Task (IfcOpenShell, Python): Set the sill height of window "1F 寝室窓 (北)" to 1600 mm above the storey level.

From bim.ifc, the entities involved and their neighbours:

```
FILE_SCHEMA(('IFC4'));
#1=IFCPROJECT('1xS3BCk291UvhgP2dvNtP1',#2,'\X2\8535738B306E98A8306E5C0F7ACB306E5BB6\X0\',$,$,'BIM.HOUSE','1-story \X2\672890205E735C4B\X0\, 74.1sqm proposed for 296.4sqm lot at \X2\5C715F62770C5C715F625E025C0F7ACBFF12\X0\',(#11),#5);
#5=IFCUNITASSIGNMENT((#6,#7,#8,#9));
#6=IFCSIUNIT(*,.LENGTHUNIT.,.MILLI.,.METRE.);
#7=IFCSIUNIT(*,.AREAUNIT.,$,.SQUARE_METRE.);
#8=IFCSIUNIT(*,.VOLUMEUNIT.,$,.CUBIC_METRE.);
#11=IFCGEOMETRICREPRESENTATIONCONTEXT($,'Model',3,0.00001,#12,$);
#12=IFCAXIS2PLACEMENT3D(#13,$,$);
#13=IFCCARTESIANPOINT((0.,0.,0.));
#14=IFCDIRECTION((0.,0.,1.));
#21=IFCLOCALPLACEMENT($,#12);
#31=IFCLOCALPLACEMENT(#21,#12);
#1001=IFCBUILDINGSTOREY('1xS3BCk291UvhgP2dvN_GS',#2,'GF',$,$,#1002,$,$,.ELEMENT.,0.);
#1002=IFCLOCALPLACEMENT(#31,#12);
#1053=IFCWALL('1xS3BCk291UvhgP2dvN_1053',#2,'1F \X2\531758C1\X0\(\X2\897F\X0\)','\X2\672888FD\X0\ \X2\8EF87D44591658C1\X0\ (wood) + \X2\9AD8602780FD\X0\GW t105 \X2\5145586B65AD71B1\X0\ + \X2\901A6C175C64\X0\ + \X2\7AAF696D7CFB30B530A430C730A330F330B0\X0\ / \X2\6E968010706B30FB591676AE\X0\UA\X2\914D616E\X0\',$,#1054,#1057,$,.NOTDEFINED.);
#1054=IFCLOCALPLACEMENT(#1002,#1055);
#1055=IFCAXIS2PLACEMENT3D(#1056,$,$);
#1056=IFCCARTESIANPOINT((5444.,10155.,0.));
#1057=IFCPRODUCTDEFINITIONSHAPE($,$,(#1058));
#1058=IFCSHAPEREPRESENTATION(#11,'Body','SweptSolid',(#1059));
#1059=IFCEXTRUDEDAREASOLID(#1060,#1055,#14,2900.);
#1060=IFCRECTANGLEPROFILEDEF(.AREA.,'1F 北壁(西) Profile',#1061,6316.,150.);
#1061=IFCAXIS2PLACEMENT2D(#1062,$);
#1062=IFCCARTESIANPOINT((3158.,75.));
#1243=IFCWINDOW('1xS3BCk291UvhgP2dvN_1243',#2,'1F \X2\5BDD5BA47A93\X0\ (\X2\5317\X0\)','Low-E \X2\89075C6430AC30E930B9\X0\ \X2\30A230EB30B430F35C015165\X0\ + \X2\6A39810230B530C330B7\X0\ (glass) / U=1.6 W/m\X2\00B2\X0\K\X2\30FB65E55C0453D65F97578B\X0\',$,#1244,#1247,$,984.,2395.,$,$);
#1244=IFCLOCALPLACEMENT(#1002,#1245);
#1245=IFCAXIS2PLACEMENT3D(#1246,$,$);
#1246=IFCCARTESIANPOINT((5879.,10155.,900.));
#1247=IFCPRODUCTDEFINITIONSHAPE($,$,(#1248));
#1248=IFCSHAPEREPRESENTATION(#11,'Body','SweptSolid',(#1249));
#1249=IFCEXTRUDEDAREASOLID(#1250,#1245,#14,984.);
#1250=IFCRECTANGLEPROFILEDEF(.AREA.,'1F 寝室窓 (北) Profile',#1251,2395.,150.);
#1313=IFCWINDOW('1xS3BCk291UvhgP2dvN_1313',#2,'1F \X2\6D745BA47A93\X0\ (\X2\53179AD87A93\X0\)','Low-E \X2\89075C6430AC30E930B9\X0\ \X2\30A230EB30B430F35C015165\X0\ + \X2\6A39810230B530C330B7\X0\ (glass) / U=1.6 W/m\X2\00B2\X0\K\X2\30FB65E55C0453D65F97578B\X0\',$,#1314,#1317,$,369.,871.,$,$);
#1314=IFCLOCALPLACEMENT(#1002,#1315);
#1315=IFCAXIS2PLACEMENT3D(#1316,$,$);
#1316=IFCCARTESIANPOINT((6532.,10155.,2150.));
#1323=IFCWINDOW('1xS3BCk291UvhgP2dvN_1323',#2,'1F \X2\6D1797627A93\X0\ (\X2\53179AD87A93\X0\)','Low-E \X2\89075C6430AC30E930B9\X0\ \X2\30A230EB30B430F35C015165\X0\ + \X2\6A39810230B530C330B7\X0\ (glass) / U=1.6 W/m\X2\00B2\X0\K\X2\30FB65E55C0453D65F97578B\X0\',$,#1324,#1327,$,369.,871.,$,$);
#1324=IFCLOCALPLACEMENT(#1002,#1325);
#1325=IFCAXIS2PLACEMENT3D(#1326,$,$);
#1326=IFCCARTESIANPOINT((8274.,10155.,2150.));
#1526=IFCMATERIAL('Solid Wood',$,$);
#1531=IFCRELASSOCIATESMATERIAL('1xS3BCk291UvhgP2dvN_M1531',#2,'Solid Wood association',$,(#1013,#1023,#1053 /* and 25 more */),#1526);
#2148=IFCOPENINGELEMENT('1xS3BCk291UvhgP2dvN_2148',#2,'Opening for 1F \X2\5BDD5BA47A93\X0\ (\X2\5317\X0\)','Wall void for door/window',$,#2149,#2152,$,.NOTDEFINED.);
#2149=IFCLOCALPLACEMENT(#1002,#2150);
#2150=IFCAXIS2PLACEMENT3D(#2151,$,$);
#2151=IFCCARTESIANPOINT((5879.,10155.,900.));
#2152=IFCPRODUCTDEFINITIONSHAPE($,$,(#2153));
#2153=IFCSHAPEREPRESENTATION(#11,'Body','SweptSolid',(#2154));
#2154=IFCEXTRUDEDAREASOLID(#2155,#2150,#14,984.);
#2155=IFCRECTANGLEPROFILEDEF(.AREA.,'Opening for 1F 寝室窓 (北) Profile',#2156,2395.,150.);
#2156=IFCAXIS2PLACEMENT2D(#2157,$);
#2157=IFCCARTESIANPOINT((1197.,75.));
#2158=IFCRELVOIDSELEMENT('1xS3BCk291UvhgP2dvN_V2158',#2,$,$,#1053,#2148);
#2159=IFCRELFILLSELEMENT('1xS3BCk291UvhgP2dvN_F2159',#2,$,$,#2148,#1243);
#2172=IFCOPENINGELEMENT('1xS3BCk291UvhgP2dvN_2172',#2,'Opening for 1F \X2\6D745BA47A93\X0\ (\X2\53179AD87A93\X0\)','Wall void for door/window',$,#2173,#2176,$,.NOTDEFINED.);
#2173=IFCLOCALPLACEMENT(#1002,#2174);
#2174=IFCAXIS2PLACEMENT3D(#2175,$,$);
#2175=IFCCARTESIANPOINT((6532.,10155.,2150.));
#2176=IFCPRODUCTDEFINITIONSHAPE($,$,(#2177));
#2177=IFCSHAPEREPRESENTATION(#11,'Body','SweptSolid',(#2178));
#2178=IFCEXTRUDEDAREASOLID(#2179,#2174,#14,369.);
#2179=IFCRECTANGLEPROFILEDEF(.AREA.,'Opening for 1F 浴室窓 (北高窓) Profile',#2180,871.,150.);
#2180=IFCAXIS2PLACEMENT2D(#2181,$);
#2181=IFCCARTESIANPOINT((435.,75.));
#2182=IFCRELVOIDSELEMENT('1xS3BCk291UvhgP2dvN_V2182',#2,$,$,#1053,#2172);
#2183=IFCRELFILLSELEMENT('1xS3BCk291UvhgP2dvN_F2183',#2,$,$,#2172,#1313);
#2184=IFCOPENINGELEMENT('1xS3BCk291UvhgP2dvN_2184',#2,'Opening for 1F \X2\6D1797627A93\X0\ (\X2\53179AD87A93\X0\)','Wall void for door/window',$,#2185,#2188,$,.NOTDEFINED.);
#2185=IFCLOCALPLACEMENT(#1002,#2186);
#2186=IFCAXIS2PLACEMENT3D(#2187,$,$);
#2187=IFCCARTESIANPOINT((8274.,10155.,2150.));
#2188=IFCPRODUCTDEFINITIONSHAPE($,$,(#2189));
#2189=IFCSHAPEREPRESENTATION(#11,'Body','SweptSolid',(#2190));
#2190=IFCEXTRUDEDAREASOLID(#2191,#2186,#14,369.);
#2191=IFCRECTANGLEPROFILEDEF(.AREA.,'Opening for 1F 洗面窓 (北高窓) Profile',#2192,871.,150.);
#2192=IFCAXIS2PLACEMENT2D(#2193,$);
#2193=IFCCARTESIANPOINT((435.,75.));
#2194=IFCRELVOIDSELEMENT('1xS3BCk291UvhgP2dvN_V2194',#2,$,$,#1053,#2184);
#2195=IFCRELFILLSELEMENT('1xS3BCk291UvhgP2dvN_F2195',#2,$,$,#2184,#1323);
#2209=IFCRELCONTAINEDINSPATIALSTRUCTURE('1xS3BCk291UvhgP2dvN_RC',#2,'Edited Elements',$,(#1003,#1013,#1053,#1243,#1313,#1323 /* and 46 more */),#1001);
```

```python
import numpy as np
import ifcopenshell
import ifcopenshell.api.geometry
import ifcopenshell.geom
import ifcopenshell.util.element
import ifcopenshell.util.placement
import ifcopenshell.util.shape
import ifcopenshell.util.unit

model = ifcopenshell.open("bim.ifc")
unit_scale = ifcopenshell.util.unit.calculate_unit_scale(model)

window = model.by_guid("1xS3BCk291UvhgP2dvN_1243")
opening = window.FillsVoids[0].RelatingOpeningElement
storey = ifcopenshell.util.element.get_container(window, ifc_class="IfcBuildingStorey")
level = ifcopenshell.util.placement.get_local_placement(storey.ObjectPlacement)[2, 3]

# The opening's origin need not be at the sill, so measure its lowest point.
shape = ifcopenshell.geom.create_shape(ifcopenshell.geom.settings(), opening)
bottom = ifcopenshell.util.shape.get_shape_bottom_elevation(shape, shape.geometry) / unit_scale
dz = level + 1600.0 - bottom

shift = np.array([0.0, 0.0, dz])
# The window is not placed relative to its opening, so move both.
for product in (opening, window):
    matrix = ifcopenshell.util.placement.get_local_placement(product.ObjectPlacement)
    matrix[:3, 3] += shift
    ifcopenshell.api.geometry.edit_object_placement(model, product=product, matrix=matrix, is_si=False)

print(f"moved by {dz * unit_scale:+.3f} m")

model.write("bim_edited.ifc")
```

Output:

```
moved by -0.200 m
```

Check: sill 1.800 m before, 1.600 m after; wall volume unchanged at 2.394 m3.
